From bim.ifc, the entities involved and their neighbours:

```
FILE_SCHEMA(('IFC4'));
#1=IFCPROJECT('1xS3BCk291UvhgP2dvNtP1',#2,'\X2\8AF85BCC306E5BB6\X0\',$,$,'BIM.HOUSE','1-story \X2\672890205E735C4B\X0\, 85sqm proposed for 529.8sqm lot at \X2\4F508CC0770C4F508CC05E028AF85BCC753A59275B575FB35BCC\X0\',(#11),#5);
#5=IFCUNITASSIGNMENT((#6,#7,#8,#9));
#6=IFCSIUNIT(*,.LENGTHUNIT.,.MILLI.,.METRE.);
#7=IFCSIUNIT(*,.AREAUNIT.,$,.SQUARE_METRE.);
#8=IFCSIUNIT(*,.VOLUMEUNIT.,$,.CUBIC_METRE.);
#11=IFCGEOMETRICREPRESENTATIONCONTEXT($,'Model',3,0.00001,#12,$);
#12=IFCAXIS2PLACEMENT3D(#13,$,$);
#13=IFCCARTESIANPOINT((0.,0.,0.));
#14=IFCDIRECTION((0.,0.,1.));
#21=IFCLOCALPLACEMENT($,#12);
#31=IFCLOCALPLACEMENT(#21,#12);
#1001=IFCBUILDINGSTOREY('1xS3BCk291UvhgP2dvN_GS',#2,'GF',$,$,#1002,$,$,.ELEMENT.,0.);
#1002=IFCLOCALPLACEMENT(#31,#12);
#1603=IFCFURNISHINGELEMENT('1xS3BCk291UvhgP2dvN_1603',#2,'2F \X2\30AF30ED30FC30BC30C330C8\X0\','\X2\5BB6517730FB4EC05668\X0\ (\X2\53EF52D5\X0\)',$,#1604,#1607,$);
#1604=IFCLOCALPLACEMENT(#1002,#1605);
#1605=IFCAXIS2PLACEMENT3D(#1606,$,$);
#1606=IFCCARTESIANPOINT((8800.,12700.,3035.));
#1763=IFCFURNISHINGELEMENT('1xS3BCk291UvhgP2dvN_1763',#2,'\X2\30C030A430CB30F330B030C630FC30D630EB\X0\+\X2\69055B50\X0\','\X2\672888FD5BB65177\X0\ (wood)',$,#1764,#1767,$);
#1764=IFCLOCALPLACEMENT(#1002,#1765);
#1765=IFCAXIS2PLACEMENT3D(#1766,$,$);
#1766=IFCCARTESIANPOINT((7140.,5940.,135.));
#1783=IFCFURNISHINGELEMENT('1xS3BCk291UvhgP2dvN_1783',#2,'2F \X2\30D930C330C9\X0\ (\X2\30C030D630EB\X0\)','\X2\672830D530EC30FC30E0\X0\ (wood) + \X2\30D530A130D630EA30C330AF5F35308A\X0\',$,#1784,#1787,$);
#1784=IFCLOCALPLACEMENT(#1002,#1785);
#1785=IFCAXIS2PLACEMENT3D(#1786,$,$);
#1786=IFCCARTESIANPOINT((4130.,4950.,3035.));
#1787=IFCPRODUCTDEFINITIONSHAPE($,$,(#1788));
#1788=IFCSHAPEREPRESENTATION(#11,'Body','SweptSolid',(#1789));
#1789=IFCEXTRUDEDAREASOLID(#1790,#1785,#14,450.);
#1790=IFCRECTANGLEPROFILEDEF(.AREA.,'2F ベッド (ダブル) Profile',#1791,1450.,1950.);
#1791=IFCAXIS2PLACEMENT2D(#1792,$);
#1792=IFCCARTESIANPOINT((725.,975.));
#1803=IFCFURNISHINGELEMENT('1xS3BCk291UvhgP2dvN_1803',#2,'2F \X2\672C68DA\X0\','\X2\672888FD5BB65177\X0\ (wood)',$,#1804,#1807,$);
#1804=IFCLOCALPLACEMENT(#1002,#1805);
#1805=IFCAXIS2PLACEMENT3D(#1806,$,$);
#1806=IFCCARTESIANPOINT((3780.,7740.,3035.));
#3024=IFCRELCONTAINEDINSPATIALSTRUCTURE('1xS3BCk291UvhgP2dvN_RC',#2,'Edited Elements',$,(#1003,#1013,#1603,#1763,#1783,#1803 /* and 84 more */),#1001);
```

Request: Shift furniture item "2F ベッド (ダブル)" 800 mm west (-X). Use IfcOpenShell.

```python
import ifcopenshell
import ifcopenshell.api.geometry
import ifcopenshell.util.placement
import ifcopenshell.util.unit

model = ifcopenshell.open("bim.ifc")
unit_scale = ifcopenshell.util.unit.calculate_unit_scale(model)

item = model.by_guid("1xS3BCk291UvhgP2dvN_1783")
matrix = ifcopenshell.util.placement.get_local_placement(item.ObjectPlacement)
matrix[0, 3] -= 0.8 / unit_scale
ifcopenshell.api.geometry.edit_object_placement(model, product=item, matrix=matrix, is_si=False)

print(ifcopenshell.util.placement.get_local_placement(item.ObjectPlacement).round(3) + 0.0)

model.write("bim_rev.ifc")
```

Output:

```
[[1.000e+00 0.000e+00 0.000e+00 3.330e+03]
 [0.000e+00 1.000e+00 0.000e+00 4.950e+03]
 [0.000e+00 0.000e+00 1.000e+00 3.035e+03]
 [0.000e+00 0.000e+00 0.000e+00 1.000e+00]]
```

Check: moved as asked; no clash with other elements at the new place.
